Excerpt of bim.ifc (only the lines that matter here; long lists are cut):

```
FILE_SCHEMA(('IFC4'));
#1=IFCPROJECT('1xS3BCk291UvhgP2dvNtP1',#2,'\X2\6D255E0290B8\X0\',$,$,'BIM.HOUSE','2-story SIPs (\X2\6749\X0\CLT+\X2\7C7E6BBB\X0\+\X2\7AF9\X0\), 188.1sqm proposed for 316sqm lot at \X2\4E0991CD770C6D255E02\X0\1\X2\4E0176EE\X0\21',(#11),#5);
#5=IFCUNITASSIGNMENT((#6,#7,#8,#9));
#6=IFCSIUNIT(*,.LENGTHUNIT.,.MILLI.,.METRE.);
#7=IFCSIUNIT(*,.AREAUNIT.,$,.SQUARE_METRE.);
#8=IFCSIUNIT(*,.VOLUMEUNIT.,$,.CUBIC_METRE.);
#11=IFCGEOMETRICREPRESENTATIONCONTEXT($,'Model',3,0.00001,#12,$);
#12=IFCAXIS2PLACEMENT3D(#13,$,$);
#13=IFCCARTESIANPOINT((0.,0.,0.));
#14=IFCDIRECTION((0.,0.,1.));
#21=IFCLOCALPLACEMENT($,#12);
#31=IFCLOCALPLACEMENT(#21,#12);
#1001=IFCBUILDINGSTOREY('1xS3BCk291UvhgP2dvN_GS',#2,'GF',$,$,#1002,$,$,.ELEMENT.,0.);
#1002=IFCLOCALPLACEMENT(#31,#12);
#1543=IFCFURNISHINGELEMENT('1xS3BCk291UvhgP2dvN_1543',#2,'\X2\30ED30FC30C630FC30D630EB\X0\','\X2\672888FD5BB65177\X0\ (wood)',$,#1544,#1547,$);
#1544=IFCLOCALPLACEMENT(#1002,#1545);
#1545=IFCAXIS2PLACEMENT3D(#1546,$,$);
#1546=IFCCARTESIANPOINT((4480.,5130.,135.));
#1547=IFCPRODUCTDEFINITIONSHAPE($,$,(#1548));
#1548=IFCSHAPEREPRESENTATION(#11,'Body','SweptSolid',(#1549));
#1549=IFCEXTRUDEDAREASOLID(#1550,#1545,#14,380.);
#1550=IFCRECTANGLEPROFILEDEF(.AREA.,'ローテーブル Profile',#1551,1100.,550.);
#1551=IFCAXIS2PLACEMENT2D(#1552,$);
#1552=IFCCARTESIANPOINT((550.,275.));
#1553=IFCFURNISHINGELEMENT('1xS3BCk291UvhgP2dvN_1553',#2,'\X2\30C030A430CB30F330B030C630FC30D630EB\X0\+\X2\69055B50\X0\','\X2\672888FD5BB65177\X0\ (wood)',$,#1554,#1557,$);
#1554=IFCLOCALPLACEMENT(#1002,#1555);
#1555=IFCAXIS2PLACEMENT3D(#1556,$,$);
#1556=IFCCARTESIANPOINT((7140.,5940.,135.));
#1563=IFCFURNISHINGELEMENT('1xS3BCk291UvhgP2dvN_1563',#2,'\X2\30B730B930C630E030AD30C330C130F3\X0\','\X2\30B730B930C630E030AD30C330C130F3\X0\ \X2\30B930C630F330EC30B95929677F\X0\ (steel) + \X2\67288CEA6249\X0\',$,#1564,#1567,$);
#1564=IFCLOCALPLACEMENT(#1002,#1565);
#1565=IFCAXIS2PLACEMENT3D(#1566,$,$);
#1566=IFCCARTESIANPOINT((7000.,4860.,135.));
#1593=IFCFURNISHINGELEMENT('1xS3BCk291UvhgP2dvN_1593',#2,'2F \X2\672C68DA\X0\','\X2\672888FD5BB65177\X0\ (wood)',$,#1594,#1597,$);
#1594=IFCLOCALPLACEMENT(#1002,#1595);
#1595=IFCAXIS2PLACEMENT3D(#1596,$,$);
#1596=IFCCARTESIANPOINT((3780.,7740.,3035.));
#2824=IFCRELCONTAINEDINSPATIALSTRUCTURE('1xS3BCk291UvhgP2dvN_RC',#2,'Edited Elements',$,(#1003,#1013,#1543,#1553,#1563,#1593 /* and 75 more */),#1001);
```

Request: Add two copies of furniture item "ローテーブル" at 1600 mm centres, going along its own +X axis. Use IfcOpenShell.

```python
import ifcopenshell
import ifcopenshell.api.geometry
import ifcopenshell.api.root
import ifcopenshell.util.element
import ifcopenshell.util.placement
import ifcopenshell.util.unit

model = ifcopenshell.open("bim.ifc")
unit_scale = ifcopenshell.util.unit.calculate_unit_scale(model)


def reuse_history(source, copy):
    """copy_class also copies each property set's owner history, people and application; keep the originals."""
    for rel in copy.IsDefinedBy:
        if rel.is_a("IfcRelDefinesByProperties") and (history := rel.RelatingPropertyDefinition.OwnerHistory):
            rel.RelatingPropertyDefinition.OwnerHistory = source.OwnerHistory
            ifcopenshell.util.element.remove_deep2(model, history)


source = model.by_guid("1xS3BCk291UvhgP2dvN_1543")
base = ifcopenshell.util.placement.get_local_placement(source.ObjectPlacement)
step = base[:3, 0] * 1.6 / unit_scale

for i in range(1, 3):
    copy = ifcopenshell.api.root.copy_class(model, product=source)
    copy.Representation = ifcopenshell.util.element.copy_deep(
        model, source.Representation, exclude=["IfcGeometricRepresentationContext", "IfcRepresentationMap"]
    )
    reuse_history(source, copy)
    matrix = base.copy()
    matrix[:3, 3] += i * step
    print("added at", matrix[:3, 3].round(3) + 0.0)
    ifcopenshell.api.geometry.edit_object_placement(model, product=copy, matrix=matrix, is_si=False)

model.write("bim-out.ifc")
```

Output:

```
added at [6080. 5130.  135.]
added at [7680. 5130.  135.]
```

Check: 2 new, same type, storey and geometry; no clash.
